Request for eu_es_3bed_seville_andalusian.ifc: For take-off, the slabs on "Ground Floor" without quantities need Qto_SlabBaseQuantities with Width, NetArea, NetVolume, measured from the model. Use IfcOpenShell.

First a look at what the model holds.

```python
import ifcopenshell
import ifcopenshell.util.element
import ifcopenshell.util.unit

model = ifcopenshell.open("eu_es_3bed_seville_andalusian.ifc")
print(model.schema)
for unit_type in ("LENGTHUNIT", "AREAUNIT", "VOLUMEUNIT"):
    print(unit_type, ifcopenshell.util.unit.calculate_unit_scale(model, unit_type))
storey = next(s for s in model.by_type("IfcBuildingStorey") if s.Name == "Ground Floor")
slabs = [e for e in ifcopenshell.util.element.get_decomposition(storey) if e.is_a("IfcSlab")]
for e in sorted(slabs, key=lambda e: e.id()):
    print(e.id(), e.is_a(), e.Name, list(ifcopenshell.util.element.get_psets(e, qtos_only=True)), sep=" | ")
```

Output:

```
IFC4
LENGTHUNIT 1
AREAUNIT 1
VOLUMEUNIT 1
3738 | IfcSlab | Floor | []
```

```python
import ifcopenshell
import ifcopenshell.api.pset
import ifcopenshell.geom
import ifcopenshell.util.element
import ifcopenshell.util.shape
import ifcopenshell.util.unit

model = ifcopenshell.open("eu_es_3bed_seville_andalusian.ifc")
unit_scale = ifcopenshell.util.unit.calculate_unit_scale(model)
area_scale = ifcopenshell.util.unit.calculate_unit_scale(model, "AREAUNIT")
volume_scale = ifcopenshell.util.unit.calculate_unit_scale(model, "VOLUMEUNIT")
settings = ifcopenshell.geom.settings()

storey = next(s for s in model.by_type("IfcBuildingStorey") if s.Name == "Ground Floor")
slabs = [e for e in ifcopenshell.util.element.get_decomposition(storey) if e.is_a("IfcSlab")]

for e in sorted(slabs, key=lambda e: e.id()):
    if ifcopenshell.util.element.get_psets(e, qtos_only=True, should_inherit=False):
        continue
    # Geometry comes back in metres, in the element's own axes.
    shape = ifcopenshell.geom.create_shape(settings, e)
    values = {
        "Width": ifcopenshell.util.shape.get_z(shape.geometry) / unit_scale,
        "NetArea": ifcopenshell.util.shape.get_footprint_area(shape.geometry) / area_scale,
        "NetVolume": ifcopenshell.util.shape.get_volume(shape.geometry) / volume_scale,
    }
    qto = ifcopenshell.api.pset.add_qto(model, product=e, name="Qto_SlabBaseQuantities")
    ifcopenshell.api.pset.edit_qto(model, qto=qto, properties=values)
    print(e.id(), {k: round(v, 3) for k, v in values.items()})

model.write("eu_es_3bed_seville_andalusian-out.ifc")
```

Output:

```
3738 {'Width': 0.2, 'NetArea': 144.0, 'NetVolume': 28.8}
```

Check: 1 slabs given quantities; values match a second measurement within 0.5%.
